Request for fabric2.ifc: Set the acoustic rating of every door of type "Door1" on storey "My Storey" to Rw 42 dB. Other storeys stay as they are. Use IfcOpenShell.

First a look at what the model holds.

```python
import ifcopenshell
import ifcopenshell.util.element

model = ifcopenshell.open("fabric2.ifc")
print(model.schema)
storey = next(s for s in model.by_type("IfcBuildingStorey") if s.Name == "My Storey")
doors = [e for e in ifcopenshell.util.element.get_decomposition(storey) if e.is_a("IfcDoor")]
seen = {}
for e in doors:
    element_type = ifcopenshell.util.element.get_type(e)
    key = (element_type.Name if element_type != e and element_type else None, ifcopenshell.util.element.get_pset(e, "Pset_DoorCommon", "AcousticRating"))
    seen[key] = seen.get(key, 0) + 1
for (name, value), count in sorted(seen.items(), key=str):
    print(count, "x", name, "|", value)
```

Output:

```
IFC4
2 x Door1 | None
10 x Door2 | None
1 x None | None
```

```python
import ifcopenshell
import ifcopenshell.api.pset
import ifcopenshell.util.element

model = ifcopenshell.open("fabric2.ifc")

storey = next(s for s in model.by_type("IfcBuildingStorey") if s.Name == "My Storey")
doors = [e for e in ifcopenshell.util.element.get_decomposition(storey) if e.is_a("IfcDoor")]

count = 0
for e in doors:
    element_type = ifcopenshell.util.element.get_type(e)
    if element_type in (None, e) or element_type.Name != "Door1":
        continue
    # add_pset returns the element's existing set when there is one.
    pset = ifcopenshell.api.pset.add_pset(model, product=e, name="Pset_DoorCommon")
    ifcopenshell.api.pset.edit_pset(model, pset=pset, properties={"AcousticRating": "Rw 42 dB"})
    count += 1

print(count, "doors updated")

model.write("fabric2_edited.ifc")
```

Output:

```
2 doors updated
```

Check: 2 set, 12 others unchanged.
